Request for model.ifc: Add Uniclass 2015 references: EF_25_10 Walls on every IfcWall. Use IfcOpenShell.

First a look at what the model holds.

```python
import ifcopenshell

model = ifcopenshell.open("model.ifc")
print(model.schema)
print("classifications:", [c.Name for c in model.by_type("IfcClassification")])
for ifc_class in ("IfcDoor", "IfcRoof", "IfcStair", "IfcWall", "IfcWindow"):
    print(ifc_class, len(model.by_type(ifc_class)))
```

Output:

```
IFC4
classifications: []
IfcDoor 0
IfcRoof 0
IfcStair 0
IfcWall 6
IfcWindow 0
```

```python
import ifcopenshell
import ifcopenshell.api.classification

model = ifcopenshell.open("model.ifc")

system = ifcopenshell.api.classification.add_classification(model, classification="Uniclass 2015")

codes = {
    "IfcWall": ("EF_25_10", "Walls"),
}
for ifc_class, (code, name) in codes.items():
    products = model.by_type(ifc_class)
    ifcopenshell.api.classification.add_reference(
        model, products=products, classification=system, identification=code, name=name
    )
    print(code, len(products))

model.write("model-out.ifc")
```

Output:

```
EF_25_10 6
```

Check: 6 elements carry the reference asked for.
